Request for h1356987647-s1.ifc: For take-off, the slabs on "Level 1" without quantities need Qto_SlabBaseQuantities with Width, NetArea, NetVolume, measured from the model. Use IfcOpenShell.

First a look at what the model holds.

```python
import ifcopenshell
import ifcopenshell.util.element
import ifcopenshell.util.unit

model = ifcopenshell.open("h1356987647-s1.ifc")
print(model.schema)
for unit_type in ("LENGTHUNIT", "AREAUNIT", "VOLUMEUNIT"):
    print(unit_type, ifcopenshell.util.unit.calculate_unit_scale(model, unit_type))
storey = next(s for s in model.by_type("IfcBuildingStorey") if s.Name == "Level 1")
slabs = [e for e in ifcopenshell.util.element.get_decomposition(storey) if e.is_a("IfcSlab")]
for e in sorted(slabs, key=lambda e: e.id()):
    print(e.id(), e.is_a(), e.Name, list(ifcopenshell.util.element.get_psets(e, qtos_only=True)), sep=" | ")
```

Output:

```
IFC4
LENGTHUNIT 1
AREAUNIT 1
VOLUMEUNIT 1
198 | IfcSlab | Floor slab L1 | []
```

```python
import ifcopenshell
import ifcopenshell.api.pset
import ifcopenshell.geom
import ifcopenshell.util.element
import ifcopenshell.util.shape
import ifcopenshell.util.unit

model = ifcopenshell.open("h1356987647-s1.ifc")
unit_scale = ifcopenshell.util.unit.calculate_unit_scale(model)
area_scale = ifcopenshell.util.unit.calculate_unit_scale(model, "AREAUNIT")
volume_scale = ifcopenshell.util.unit.calculate_unit_scale(model, "VOLUMEUNIT")
settings = ifcopenshell.geom.settings()

storey = next(s for s in model.by_type("IfcBuildingStorey") if s.Name == "Level 1")
slabs = [e for e in ifcopenshell.util.element.get_decomposition(storey) if e.is_a("IfcSlab")]

for e in sorted(slabs, key=lambda e: e.id()):
    if ifcopenshell.util.element.get_psets(e, qtos_only=True, should_inherit=False):
        continue
    # Geometry comes back in metres, in the element's own axes.
    shape = ifcopenshell.geom.create_shape(settings, e)
    values = {
        "Width": ifcopenshell.util.shape.get_z(shape.geometry) / unit_scale,
        "NetArea": ifcopenshell.util.shape.get_footprint_area(shape.geometry) / area_scale,
        "NetVolume": ifcopenshell.util.shape.get_volume(shape.geometry) / volume_scale,
    }
    qto = ifcopenshell.api.pset.add_qto(model, product=e, name="Qto_SlabBaseQuantities")
    ifcopenshell.api.pset.edit_qto(model, qto=qto, properties=values)
    print(e.id(), {k: round(v, 3) for k, v in values.items()})

model.write("h1356987647-s1_v2.ifc")
```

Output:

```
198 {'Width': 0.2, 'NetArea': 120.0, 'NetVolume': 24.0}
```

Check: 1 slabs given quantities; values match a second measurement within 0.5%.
